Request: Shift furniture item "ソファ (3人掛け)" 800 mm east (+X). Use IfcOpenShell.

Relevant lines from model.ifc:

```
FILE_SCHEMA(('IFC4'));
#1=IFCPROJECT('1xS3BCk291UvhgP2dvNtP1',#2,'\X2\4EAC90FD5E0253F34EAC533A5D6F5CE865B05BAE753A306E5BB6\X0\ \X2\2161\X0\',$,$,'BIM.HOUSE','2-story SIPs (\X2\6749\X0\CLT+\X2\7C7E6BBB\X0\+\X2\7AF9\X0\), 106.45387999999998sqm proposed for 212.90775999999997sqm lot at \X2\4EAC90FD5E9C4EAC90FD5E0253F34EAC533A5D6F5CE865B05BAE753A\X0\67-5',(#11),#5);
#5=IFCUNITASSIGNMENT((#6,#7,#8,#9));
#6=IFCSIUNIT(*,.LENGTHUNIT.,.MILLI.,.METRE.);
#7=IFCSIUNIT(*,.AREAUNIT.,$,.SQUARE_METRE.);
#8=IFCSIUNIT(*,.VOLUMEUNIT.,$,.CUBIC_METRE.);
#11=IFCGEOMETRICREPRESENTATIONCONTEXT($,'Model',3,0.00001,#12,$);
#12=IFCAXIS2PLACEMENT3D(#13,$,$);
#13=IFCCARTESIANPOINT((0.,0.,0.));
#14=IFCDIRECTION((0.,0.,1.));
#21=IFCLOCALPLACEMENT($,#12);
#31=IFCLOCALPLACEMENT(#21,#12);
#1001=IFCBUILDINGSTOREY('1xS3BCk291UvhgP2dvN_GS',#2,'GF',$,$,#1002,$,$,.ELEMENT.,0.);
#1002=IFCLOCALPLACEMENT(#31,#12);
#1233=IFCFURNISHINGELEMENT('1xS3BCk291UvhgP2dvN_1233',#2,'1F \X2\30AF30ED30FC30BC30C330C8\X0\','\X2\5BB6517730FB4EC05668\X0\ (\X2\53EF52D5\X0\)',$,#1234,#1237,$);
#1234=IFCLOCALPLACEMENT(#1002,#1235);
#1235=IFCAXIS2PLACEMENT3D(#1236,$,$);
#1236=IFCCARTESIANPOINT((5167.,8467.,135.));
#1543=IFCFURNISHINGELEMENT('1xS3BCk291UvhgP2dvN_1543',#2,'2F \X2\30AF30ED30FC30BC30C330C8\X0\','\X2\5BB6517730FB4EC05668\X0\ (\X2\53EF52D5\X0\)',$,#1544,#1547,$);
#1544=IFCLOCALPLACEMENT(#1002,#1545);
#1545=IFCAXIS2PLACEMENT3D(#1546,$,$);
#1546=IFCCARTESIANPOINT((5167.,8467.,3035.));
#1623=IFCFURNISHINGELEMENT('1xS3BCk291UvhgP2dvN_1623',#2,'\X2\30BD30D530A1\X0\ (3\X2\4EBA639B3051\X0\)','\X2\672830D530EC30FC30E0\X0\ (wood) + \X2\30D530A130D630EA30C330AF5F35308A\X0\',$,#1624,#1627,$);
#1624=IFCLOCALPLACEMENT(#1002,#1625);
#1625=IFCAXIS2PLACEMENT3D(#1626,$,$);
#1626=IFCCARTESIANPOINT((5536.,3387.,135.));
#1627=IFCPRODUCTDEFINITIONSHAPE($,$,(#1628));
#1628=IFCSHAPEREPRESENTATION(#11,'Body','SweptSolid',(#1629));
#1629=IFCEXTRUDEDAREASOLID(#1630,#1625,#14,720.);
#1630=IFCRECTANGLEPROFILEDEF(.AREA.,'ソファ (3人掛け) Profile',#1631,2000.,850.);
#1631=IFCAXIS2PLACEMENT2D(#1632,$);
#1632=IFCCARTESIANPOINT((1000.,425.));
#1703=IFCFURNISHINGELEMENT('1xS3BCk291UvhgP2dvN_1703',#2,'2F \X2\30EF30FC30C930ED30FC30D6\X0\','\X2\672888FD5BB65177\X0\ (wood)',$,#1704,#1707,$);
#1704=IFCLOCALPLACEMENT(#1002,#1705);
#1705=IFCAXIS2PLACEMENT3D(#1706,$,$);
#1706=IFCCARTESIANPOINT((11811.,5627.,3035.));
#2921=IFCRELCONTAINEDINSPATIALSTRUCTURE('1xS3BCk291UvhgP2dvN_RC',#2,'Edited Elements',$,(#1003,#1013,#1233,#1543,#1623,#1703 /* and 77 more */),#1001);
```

```python
import ifcopenshell
import ifcopenshell.api.geometry
import ifcopenshell.util.placement

model = ifcopenshell.open("model.ifc")

item = model.by_id(1623)
matrix = ifcopenshell.util.placement.get_local_placement(item.ObjectPlacement)
matrix[0, 3] += 800.0
ifcopenshell.api.geometry.edit_object_placement(model, product=item, matrix=matrix, is_si=False)

print(ifcopenshell.util.placement.get_local_placement(item.ObjectPlacement).round(3) + 0.0)

model.write("model_rev.ifc")
```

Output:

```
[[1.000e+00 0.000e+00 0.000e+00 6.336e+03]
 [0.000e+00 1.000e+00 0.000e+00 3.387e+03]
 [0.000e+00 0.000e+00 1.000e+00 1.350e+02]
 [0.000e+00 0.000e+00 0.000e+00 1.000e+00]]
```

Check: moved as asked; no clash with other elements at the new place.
